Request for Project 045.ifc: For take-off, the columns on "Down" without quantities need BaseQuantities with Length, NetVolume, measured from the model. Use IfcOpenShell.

First a look at what the model holds.

```python
import ifcopenshell
import ifcopenshell.util.element
import ifcopenshell.util.unit

model = ifcopenshell.open("Project 045.ifc")
print(model.schema)
for unit_type in ("LENGTHUNIT", "AREAUNIT", "VOLUMEUNIT"):
    print(unit_type, ifcopenshell.util.unit.calculate_unit_scale(model, unit_type))
storey = next(s for s in model.by_type("IfcBuildingStorey") if s.Name == "Down")
columns = [e for e in ifcopenshell.util.element.get_decomposition(storey) if e.is_a("IfcColumn")]
for e in sorted(columns, key=lambda e: e.id()):
    print(e.id(), e.is_a(), e.Name, list(ifcopenshell.util.element.get_psets(e, qtos_only=True)), sep=" | ")
```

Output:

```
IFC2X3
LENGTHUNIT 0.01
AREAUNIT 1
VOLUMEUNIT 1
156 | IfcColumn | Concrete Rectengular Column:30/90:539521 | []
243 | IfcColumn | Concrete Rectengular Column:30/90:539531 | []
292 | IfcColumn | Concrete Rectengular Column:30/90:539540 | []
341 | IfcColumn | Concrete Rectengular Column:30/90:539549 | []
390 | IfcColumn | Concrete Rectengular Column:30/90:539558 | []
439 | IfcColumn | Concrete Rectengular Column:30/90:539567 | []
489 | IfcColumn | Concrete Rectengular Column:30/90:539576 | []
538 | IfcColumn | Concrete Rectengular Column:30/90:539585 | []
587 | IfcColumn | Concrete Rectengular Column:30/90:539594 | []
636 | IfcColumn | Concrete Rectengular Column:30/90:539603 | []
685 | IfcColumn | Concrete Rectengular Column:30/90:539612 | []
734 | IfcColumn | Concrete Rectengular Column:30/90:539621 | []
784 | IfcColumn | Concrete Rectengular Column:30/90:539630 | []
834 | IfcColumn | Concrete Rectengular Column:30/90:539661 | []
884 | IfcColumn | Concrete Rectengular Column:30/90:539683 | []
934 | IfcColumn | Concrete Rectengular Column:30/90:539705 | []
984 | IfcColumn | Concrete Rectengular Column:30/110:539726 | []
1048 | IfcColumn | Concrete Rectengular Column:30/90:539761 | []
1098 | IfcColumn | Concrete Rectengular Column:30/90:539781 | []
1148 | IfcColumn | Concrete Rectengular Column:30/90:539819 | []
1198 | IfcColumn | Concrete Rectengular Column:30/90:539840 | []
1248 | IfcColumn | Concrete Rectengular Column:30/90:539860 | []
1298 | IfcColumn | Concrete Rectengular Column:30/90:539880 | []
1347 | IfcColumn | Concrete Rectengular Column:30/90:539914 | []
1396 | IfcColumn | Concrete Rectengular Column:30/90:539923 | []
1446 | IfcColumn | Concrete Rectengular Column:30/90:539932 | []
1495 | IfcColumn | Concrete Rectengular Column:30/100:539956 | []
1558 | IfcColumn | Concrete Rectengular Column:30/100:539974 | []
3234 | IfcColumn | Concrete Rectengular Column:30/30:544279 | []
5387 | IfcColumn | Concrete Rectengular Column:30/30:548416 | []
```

```python
import ifcopenshell
import ifcopenshell.api.pset
import ifcopenshell.geom
import ifcopenshell.util.element
import ifcopenshell.util.shape
import ifcopenshell.util.unit

model = ifcopenshell.open("Project 045.ifc")
unit_scale = ifcopenshell.util.unit.calculate_unit_scale(model)
volume_scale = ifcopenshell.util.unit.calculate_unit_scale(model, "VOLUMEUNIT")
settings = ifcopenshell.geom.settings()

storey = next(s for s in model.by_type("IfcBuildingStorey") if s.Name == "Down")
columns = [e for e in ifcopenshell.util.element.get_decomposition(storey) if e.is_a("IfcColumn")]

for e in sorted(columns, key=lambda e: e.id()):
    if ifcopenshell.util.element.get_psets(e, qtos_only=True, should_inherit=False):
        continue
    # Geometry comes back in metres, in the element's own axes.
    shape = ifcopenshell.geom.create_shape(settings, e)
    values = {
        "Length": ifcopenshell.util.shape.get_z(shape.geometry) / unit_scale,
        "NetVolume": ifcopenshell.util.shape.get_volume(shape.geometry) / volume_scale,
    }
    qto = ifcopenshell.api.pset.add_qto(model, product=e, name="BaseQuantities")
    ifcopenshell.api.pset.edit_qto(model, qto=qto, properties=values)
    print(e.id(), {k: round(v, 3) for k, v in values.items()})

model.write("Project 045_v2.ifc")
```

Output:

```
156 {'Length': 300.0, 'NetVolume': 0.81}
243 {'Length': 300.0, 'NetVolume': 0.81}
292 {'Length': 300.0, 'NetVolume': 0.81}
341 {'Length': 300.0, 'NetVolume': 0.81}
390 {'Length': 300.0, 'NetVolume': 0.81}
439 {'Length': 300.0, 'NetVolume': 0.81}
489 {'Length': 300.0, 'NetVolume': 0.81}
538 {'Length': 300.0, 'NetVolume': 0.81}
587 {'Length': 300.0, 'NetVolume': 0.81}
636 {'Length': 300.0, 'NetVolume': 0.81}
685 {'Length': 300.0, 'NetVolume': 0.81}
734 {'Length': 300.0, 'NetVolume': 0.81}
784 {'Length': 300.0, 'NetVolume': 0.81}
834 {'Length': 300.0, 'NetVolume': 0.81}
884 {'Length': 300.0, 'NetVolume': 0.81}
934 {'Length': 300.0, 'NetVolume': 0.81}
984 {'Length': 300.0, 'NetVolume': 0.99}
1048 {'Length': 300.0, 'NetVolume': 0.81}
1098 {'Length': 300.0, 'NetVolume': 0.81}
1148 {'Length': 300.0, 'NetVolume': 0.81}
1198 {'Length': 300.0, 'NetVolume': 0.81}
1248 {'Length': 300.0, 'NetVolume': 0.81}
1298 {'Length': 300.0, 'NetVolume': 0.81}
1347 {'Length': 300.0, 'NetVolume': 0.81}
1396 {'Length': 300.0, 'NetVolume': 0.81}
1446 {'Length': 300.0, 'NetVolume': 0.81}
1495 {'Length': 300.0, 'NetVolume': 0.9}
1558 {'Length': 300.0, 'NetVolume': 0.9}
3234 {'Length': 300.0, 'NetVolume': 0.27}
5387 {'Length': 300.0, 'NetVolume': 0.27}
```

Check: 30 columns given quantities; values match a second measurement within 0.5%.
